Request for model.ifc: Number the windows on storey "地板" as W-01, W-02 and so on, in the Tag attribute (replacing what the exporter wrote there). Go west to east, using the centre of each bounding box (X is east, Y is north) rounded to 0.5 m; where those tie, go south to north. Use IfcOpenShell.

First a look at what the model holds.

```python
import ifcopenshell
import ifcopenshell.util.element
import ifcopenshell.util.placement

model = ifcopenshell.open("model.ifc")
print(model.schema)
storey = next(s for s in model.by_type("IfcBuildingStorey") if s.Name == "地板")
windows = [e for e in ifcopenshell.util.element.get_decomposition(storey) if e.is_a("IfcWindow")]
for e in sorted(windows, key=lambda e: e.id()):
    origin = ifcopenshell.util.placement.get_local_placement(e.ObjectPlacement)[:3, 3]
    print(e.id(), e.Tag, e.Name, origin.round(2) + 0.0, sep=" | ")
```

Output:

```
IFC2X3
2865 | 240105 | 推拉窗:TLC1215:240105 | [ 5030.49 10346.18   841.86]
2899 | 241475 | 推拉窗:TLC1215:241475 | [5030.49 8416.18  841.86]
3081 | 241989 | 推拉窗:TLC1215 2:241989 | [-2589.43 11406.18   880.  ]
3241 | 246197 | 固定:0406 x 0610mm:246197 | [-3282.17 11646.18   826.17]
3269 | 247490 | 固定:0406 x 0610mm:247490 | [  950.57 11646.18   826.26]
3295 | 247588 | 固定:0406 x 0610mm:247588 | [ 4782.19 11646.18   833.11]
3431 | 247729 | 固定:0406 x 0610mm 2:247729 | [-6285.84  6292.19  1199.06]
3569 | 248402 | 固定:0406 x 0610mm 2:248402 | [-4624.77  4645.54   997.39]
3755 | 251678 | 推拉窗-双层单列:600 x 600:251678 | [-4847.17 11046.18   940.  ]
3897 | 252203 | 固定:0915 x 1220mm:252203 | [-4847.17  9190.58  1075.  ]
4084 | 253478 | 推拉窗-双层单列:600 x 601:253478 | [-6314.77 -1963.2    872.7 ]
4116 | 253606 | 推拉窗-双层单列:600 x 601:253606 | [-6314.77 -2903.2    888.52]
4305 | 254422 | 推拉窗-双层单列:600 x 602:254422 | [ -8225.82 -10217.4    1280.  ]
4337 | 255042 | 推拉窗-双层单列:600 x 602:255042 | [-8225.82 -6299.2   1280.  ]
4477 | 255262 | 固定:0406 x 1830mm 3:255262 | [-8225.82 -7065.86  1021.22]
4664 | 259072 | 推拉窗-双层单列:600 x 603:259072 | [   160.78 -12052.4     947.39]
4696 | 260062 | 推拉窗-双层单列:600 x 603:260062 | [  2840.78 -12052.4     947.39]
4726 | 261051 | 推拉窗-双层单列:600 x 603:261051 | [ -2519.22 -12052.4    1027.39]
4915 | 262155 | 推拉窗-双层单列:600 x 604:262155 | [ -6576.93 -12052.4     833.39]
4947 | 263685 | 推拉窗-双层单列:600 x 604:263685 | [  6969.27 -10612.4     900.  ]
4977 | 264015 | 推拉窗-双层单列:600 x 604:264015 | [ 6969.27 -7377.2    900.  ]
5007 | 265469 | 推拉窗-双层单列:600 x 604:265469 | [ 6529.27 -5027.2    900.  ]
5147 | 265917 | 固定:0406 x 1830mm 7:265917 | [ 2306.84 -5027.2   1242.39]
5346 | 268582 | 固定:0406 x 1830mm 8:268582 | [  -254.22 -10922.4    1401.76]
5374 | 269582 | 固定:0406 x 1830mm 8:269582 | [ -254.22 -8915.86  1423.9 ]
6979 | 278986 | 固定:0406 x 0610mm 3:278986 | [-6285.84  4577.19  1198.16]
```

```python
import ifcopenshell
import ifcopenshell.geom
import ifcopenshell.util.element
import ifcopenshell.util.shape

model = ifcopenshell.open("model.ifc")
settings = ifcopenshell.geom.settings()
settings.set("use-world-coords", True)


def centre(element):
    shape = ifcopenshell.geom.create_shape(settings, element)
    return ifcopenshell.util.shape.get_bbox_centroid(shape.geometry)


storey = next(s for s in model.by_type("IfcBuildingStorey") if s.Name == "地板")
windows = [e for e in ifcopenshell.util.element.get_decomposition(storey) if e.is_a("IfcWindow")]

# Insertion points can sit at a corner or the storey origin, so sort by the geometry (in metres).
centres = {e: centre(e) for e in windows}
windows.sort(key=lambda e: (round(centres[e][0] / 0.5), centres[e][1]))

for i, e in enumerate(windows, start=1):
    number = f"W-{i:02d}"
    e.Tag = number
    print(e.id(), number)

model.write("model_updated.ifc")
```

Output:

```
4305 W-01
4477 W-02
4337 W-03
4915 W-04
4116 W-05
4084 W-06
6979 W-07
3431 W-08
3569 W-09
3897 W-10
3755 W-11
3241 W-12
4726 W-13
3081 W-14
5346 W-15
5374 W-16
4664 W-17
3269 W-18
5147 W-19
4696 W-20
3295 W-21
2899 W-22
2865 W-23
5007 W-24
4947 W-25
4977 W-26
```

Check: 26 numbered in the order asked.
